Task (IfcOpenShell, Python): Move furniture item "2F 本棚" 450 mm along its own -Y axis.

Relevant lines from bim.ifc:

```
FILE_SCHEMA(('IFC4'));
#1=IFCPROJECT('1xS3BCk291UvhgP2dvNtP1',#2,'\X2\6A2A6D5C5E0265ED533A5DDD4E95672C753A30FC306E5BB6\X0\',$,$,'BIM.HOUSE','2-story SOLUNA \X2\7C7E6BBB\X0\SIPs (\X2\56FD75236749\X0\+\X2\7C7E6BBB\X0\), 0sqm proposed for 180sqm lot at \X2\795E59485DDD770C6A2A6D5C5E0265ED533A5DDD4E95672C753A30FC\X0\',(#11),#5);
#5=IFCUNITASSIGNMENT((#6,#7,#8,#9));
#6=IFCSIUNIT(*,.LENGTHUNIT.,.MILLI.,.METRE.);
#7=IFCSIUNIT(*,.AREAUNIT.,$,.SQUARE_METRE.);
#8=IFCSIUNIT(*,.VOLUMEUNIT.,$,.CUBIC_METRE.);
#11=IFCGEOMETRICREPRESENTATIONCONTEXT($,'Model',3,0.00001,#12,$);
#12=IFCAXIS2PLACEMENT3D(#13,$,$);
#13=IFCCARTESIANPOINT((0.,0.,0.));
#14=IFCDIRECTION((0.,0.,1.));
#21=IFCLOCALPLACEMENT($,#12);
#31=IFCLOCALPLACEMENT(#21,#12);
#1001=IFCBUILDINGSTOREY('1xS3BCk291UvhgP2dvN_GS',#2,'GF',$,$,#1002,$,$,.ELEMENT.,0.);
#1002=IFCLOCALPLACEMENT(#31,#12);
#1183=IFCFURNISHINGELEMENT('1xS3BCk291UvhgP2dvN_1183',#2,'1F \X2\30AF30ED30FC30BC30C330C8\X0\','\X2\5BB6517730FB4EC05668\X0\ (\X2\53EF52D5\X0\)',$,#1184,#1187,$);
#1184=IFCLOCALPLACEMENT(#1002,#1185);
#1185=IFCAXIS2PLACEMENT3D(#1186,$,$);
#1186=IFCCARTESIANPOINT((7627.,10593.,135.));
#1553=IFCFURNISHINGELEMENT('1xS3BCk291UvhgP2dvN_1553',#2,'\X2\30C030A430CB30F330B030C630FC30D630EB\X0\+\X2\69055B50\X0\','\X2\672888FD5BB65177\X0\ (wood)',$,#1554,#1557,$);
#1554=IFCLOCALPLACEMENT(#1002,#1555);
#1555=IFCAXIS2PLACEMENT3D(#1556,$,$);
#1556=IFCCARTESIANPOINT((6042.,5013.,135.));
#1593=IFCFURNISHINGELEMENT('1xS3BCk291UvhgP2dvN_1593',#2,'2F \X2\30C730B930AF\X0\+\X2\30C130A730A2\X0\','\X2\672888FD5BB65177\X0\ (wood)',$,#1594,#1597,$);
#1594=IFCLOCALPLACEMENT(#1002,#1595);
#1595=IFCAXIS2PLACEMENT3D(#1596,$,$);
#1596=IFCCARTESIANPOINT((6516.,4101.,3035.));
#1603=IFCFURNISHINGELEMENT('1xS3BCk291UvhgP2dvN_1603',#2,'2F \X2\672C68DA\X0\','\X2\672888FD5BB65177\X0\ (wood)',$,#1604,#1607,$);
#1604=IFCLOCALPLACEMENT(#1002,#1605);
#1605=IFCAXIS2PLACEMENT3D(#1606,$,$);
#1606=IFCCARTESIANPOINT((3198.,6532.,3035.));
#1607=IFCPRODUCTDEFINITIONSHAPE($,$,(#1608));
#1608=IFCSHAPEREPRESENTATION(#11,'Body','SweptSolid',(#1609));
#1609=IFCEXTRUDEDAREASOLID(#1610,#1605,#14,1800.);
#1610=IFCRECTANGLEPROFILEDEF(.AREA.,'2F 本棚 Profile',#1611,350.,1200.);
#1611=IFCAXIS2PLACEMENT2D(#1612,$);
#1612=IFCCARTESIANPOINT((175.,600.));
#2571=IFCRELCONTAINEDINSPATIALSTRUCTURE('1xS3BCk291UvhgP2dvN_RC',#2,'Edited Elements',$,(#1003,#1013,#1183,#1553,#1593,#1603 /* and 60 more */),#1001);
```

```python
import ifcopenshell
import ifcopenshell.api.geometry
import ifcopenshell.util.placement

model = ifcopenshell.open("bim.ifc")

item = model.by_guid("1xS3BCk291UvhgP2dvN_1603")
matrix = ifcopenshell.util.placement.get_local_placement(item.ObjectPlacement)
matrix[:3, 3] -= matrix[:3, 1] * 450.0
ifcopenshell.api.geometry.edit_object_placement(model, product=item, matrix=matrix, is_si=False)

print(ifcopenshell.util.placement.get_local_placement(item.ObjectPlacement).round(3) + 0.0)

model.write("bim_rev.ifc")
```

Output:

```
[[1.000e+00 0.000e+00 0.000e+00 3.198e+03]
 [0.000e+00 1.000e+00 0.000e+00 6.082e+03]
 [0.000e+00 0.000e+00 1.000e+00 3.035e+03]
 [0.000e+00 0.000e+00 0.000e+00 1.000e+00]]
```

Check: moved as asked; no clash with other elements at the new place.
